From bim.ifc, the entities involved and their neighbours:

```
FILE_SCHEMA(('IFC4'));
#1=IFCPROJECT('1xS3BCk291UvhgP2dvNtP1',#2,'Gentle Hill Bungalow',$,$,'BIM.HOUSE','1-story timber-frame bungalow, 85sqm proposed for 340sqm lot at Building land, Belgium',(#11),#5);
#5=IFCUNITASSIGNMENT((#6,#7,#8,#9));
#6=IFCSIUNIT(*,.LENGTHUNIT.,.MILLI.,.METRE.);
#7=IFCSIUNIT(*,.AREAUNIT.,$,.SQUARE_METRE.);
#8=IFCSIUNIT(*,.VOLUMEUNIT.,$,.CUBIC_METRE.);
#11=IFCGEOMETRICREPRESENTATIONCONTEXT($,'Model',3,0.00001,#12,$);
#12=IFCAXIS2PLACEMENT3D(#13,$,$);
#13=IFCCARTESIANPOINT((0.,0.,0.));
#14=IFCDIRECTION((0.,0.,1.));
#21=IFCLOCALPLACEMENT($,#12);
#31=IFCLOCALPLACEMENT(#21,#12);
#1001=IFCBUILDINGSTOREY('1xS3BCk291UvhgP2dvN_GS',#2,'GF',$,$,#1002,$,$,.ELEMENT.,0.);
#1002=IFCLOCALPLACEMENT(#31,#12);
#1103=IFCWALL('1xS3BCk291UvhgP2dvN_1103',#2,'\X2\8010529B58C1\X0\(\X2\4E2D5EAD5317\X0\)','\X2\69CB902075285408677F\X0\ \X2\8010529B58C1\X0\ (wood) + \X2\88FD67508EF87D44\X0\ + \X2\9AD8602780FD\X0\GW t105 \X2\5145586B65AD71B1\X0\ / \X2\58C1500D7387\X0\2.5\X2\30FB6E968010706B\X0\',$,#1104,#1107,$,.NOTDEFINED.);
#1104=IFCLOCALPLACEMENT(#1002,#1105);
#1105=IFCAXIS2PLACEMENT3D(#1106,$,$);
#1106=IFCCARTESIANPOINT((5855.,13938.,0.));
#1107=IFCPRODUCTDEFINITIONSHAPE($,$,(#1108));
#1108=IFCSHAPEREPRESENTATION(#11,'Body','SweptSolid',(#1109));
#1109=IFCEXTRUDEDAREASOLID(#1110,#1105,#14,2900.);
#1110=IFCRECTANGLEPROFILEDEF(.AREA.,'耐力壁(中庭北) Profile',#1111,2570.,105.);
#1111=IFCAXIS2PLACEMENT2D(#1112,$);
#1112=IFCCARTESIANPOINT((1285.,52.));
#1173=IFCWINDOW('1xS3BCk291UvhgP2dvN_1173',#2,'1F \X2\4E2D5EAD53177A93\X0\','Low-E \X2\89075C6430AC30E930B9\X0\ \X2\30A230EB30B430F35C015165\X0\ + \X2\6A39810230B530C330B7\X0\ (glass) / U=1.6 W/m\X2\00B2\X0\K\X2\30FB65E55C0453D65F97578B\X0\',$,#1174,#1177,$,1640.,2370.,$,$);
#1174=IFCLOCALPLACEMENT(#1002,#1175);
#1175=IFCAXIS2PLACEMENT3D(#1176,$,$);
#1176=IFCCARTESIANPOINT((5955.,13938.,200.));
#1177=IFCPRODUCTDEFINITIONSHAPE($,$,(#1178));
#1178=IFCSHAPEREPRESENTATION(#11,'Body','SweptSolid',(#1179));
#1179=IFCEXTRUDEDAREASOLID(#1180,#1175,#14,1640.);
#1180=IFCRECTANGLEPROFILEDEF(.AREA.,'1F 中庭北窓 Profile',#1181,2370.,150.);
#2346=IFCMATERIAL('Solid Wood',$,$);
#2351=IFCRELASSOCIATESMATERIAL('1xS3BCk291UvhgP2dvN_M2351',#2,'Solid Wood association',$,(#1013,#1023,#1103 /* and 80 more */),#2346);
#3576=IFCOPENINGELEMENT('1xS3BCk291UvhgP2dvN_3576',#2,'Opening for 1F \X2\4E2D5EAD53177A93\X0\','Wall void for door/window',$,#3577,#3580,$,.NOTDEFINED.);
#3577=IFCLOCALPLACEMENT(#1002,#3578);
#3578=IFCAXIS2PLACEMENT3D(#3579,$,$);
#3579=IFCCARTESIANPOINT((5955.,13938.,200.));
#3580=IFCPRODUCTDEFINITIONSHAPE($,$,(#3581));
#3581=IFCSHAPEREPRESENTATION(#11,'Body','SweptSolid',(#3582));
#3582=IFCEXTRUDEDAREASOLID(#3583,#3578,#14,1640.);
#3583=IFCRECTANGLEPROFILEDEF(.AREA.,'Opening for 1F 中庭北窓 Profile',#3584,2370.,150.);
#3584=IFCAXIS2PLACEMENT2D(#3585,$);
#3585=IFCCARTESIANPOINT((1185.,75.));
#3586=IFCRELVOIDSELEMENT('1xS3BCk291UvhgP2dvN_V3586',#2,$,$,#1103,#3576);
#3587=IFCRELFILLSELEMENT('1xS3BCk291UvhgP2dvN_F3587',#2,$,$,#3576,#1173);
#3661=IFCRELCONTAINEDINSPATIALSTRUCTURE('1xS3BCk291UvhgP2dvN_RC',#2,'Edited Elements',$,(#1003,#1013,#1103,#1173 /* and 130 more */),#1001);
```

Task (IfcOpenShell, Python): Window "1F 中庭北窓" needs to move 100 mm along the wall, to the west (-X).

```python
import ifcopenshell
import ifcopenshell.api.geometry
import ifcopenshell.util.placement
import ifcopenshell.util.unit

model = ifcopenshell.open("bim.ifc")
unit_scale = ifcopenshell.util.unit.calculate_unit_scale(model)

window = model.by_id(1173)
opening = window.FillsVoids[0].RelatingOpeningElement
wall = opening.VoidsElements[0].RelatingBuildingElement

wall_matrix = ifcopenshell.util.placement.get_local_placement(wall.ObjectPlacement)
shift = wall_matrix[:3, 0] * -0.1 / unit_scale
before = ifcopenshell.util.placement.get_local_placement(window.ObjectPlacement)[:3, 3].copy()

# The window is not placed relative to its opening, so move both.
for product in (opening, window):
    matrix = ifcopenshell.util.placement.get_local_placement(product.ObjectPlacement)
    matrix[:3, 3] += shift
    ifcopenshell.api.geometry.edit_object_placement(model, product=product, matrix=matrix, is_si=False)

after = ifcopenshell.util.placement.get_local_placement(window.ObjectPlacement)[:3, 3]
print("window moved by", (after - before).round(3) + 0.0)

model.write("bim_rev.ifc")
```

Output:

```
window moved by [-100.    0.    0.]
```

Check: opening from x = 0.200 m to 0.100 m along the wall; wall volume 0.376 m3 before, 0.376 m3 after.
